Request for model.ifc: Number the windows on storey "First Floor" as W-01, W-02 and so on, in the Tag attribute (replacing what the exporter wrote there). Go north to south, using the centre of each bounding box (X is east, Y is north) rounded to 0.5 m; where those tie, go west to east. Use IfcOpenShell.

First a look at what the model holds.

```python
import ifcopenshell
import ifcopenshell.util.element
import ifcopenshell.util.placement

model = ifcopenshell.open("model.ifc")
print(model.schema)
storey = next(s for s in model.by_type("IfcBuildingStorey") if s.Name == "First Floor")
windows = [e for e in ifcopenshell.util.element.get_decomposition(storey) if e.is_a("IfcWindow")]
for e in sorted(windows, key=lambda e: e.id()):
    origin = ifcopenshell.util.placement.get_local_placement(e.ObjectPlacement)[:3, 3]
    print(e.id(), e.Tag, e.Name, origin.round(2) + 0.0, sep=" | ")
```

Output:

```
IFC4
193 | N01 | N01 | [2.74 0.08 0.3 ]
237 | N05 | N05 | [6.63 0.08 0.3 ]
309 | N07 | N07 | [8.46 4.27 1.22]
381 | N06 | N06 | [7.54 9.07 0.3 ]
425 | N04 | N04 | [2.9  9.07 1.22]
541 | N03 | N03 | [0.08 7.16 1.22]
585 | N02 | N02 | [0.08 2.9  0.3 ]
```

```python
import ifcopenshell
import ifcopenshell.geom
import ifcopenshell.util.element
import ifcopenshell.util.shape

model = ifcopenshell.open("model.ifc")
settings = ifcopenshell.geom.settings()
settings.set("use-world-coords", True)


def centre(element):
    shape = ifcopenshell.geom.create_shape(settings, element)
    return ifcopenshell.util.shape.get_bbox_centroid(shape.geometry)


storey = next(s for s in model.by_type("IfcBuildingStorey") if s.Name == "First Floor")
windows = [e for e in ifcopenshell.util.element.get_decomposition(storey) if e.is_a("IfcWindow")]

# Insertion points can sit at a corner or the storey origin, so sort by the geometry (in metres).
centres = {e: centre(e) for e in windows}
windows.sort(key=lambda e: (-round(centres[e][1] / 0.5), centres[e][0]))

for i, e in enumerate(windows, start=1):
    number = f"W-{i:02d}"
    e.Tag = number
    print(e.id(), number)

model.write("model_rev.ifc")
```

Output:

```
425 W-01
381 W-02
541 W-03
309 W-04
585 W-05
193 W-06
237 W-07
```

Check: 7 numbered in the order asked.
